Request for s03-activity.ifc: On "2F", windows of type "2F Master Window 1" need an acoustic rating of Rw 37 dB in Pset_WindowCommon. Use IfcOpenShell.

First a look at what the model holds.

```python
import ifcopenshell
import ifcopenshell.util.element

model = ifcopenshell.open("s03-activity.ifc")
print(model.schema)
storey = next(s for s in model.by_type("IfcBuildingStorey") if s.Name == "2F")
windows = [e for e in ifcopenshell.util.element.get_decomposition(storey) if e.is_a("IfcWindow")]
seen = {}
for e in windows:
    element_type = ifcopenshell.util.element.get_type(e)
    key = (element_type.Name if element_type != e and element_type else None, ifcopenshell.util.element.get_pset(e, "Pset_WindowCommon", "AcousticRating"))
    seen[key] = seen.get(key, 0) + 1
for (name, value), count in sorted(seen.items(), key=str):
    print(count, "x", name, "|", value)
```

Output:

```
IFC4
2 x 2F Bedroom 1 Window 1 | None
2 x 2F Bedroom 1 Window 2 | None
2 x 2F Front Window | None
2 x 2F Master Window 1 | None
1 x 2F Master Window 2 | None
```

```python
import ifcopenshell
import ifcopenshell.api.pset
import ifcopenshell.util.element

model = ifcopenshell.open("s03-activity.ifc")

storey = next(s for s in model.by_type("IfcBuildingStorey") if s.Name == "2F")
windows = [e for e in ifcopenshell.util.element.get_decomposition(storey) if e.is_a("IfcWindow")]

count = 0
for e in windows:
    element_type = ifcopenshell.util.element.get_type(e)
    if element_type in (None, e) or element_type.Name != "2F Master Window 1":
        continue
    # add_pset returns the element's existing set when there is one.
    pset = ifcopenshell.api.pset.add_pset(model, product=e, name="Pset_WindowCommon")
    ifcopenshell.api.pset.edit_pset(model, pset=pset, properties={"AcousticRating": "Rw 37 dB"})
    count += 1

print(count, "windows updated")

model.write("s03-activity_edited.ifc")
```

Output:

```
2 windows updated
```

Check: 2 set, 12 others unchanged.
